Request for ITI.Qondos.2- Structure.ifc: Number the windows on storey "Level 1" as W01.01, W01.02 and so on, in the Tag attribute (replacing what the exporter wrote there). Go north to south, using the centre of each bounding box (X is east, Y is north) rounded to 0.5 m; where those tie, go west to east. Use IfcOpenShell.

First a look at what the model holds.

```python
import ifcopenshell
import ifcopenshell.util.element
import ifcopenshell.util.placement

model = ifcopenshell.open("ITI.Qondos.2- Structure.ifc")
print(model.schema)
storey = next(s for s in model.by_type("IfcBuildingStorey") if s.Name == "Level 1")
windows = [e for e in ifcopenshell.util.element.get_decomposition(storey) if e.is_a("IfcWindow")]
for e in sorted(windows, key=lambda e: e.id()):
    origin = ifcopenshell.util.placement.get_local_placement(e.ObjectPlacement)[:3, 3]
    print(e.id(), e.Tag, e.Name, origin.round(2) + 0.0, sep=" | ")
```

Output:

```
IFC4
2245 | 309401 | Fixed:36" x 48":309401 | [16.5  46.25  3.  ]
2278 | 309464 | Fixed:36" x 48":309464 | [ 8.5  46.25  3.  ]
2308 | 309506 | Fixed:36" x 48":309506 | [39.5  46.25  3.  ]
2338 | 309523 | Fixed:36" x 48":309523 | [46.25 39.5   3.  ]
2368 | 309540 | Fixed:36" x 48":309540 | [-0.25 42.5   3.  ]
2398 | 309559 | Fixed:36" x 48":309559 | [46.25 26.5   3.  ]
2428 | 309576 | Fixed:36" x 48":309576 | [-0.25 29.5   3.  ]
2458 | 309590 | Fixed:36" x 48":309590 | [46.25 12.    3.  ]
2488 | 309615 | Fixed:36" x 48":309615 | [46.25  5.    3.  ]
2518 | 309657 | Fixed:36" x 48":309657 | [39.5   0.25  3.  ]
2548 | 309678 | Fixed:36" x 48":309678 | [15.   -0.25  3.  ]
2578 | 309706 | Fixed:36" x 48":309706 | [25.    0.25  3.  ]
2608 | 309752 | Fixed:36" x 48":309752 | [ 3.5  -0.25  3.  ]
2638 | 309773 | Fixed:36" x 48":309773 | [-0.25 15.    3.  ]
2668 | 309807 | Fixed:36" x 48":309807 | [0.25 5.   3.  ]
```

```python
import ifcopenshell
import ifcopenshell.geom
import ifcopenshell.util.element
import ifcopenshell.util.shape

model = ifcopenshell.open("ITI.Qondos.2- Structure.ifc")
settings = ifcopenshell.geom.settings()
settings.set("use-world-coords", True)


def centre(element):
    shape = ifcopenshell.geom.create_shape(settings, element)
    return ifcopenshell.util.shape.get_bbox_centroid(shape.geometry)


storey = next(s for s in model.by_type("IfcBuildingStorey") if s.Name == "Level 1")
windows = [e for e in ifcopenshell.util.element.get_decomposition(storey) if e.is_a("IfcWindow")]

# Insertion points can sit at a corner or the storey origin, so sort by the geometry (in metres).
centres = {e: centre(e) for e in windows}
windows.sort(key=lambda e: (-round(centres[e][1] / 0.5), centres[e][0]))

for i, e in enumerate(windows, start=1):
    number = f"W01.{i:02d}"
    e.Tag = number
    print(e.id(), number)

model.write("ITI.Qondos.2- Structure_edited.ifc")
```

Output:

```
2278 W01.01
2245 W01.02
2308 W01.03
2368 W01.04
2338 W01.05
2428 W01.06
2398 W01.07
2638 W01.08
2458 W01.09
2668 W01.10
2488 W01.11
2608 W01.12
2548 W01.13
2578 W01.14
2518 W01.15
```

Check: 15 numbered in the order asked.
